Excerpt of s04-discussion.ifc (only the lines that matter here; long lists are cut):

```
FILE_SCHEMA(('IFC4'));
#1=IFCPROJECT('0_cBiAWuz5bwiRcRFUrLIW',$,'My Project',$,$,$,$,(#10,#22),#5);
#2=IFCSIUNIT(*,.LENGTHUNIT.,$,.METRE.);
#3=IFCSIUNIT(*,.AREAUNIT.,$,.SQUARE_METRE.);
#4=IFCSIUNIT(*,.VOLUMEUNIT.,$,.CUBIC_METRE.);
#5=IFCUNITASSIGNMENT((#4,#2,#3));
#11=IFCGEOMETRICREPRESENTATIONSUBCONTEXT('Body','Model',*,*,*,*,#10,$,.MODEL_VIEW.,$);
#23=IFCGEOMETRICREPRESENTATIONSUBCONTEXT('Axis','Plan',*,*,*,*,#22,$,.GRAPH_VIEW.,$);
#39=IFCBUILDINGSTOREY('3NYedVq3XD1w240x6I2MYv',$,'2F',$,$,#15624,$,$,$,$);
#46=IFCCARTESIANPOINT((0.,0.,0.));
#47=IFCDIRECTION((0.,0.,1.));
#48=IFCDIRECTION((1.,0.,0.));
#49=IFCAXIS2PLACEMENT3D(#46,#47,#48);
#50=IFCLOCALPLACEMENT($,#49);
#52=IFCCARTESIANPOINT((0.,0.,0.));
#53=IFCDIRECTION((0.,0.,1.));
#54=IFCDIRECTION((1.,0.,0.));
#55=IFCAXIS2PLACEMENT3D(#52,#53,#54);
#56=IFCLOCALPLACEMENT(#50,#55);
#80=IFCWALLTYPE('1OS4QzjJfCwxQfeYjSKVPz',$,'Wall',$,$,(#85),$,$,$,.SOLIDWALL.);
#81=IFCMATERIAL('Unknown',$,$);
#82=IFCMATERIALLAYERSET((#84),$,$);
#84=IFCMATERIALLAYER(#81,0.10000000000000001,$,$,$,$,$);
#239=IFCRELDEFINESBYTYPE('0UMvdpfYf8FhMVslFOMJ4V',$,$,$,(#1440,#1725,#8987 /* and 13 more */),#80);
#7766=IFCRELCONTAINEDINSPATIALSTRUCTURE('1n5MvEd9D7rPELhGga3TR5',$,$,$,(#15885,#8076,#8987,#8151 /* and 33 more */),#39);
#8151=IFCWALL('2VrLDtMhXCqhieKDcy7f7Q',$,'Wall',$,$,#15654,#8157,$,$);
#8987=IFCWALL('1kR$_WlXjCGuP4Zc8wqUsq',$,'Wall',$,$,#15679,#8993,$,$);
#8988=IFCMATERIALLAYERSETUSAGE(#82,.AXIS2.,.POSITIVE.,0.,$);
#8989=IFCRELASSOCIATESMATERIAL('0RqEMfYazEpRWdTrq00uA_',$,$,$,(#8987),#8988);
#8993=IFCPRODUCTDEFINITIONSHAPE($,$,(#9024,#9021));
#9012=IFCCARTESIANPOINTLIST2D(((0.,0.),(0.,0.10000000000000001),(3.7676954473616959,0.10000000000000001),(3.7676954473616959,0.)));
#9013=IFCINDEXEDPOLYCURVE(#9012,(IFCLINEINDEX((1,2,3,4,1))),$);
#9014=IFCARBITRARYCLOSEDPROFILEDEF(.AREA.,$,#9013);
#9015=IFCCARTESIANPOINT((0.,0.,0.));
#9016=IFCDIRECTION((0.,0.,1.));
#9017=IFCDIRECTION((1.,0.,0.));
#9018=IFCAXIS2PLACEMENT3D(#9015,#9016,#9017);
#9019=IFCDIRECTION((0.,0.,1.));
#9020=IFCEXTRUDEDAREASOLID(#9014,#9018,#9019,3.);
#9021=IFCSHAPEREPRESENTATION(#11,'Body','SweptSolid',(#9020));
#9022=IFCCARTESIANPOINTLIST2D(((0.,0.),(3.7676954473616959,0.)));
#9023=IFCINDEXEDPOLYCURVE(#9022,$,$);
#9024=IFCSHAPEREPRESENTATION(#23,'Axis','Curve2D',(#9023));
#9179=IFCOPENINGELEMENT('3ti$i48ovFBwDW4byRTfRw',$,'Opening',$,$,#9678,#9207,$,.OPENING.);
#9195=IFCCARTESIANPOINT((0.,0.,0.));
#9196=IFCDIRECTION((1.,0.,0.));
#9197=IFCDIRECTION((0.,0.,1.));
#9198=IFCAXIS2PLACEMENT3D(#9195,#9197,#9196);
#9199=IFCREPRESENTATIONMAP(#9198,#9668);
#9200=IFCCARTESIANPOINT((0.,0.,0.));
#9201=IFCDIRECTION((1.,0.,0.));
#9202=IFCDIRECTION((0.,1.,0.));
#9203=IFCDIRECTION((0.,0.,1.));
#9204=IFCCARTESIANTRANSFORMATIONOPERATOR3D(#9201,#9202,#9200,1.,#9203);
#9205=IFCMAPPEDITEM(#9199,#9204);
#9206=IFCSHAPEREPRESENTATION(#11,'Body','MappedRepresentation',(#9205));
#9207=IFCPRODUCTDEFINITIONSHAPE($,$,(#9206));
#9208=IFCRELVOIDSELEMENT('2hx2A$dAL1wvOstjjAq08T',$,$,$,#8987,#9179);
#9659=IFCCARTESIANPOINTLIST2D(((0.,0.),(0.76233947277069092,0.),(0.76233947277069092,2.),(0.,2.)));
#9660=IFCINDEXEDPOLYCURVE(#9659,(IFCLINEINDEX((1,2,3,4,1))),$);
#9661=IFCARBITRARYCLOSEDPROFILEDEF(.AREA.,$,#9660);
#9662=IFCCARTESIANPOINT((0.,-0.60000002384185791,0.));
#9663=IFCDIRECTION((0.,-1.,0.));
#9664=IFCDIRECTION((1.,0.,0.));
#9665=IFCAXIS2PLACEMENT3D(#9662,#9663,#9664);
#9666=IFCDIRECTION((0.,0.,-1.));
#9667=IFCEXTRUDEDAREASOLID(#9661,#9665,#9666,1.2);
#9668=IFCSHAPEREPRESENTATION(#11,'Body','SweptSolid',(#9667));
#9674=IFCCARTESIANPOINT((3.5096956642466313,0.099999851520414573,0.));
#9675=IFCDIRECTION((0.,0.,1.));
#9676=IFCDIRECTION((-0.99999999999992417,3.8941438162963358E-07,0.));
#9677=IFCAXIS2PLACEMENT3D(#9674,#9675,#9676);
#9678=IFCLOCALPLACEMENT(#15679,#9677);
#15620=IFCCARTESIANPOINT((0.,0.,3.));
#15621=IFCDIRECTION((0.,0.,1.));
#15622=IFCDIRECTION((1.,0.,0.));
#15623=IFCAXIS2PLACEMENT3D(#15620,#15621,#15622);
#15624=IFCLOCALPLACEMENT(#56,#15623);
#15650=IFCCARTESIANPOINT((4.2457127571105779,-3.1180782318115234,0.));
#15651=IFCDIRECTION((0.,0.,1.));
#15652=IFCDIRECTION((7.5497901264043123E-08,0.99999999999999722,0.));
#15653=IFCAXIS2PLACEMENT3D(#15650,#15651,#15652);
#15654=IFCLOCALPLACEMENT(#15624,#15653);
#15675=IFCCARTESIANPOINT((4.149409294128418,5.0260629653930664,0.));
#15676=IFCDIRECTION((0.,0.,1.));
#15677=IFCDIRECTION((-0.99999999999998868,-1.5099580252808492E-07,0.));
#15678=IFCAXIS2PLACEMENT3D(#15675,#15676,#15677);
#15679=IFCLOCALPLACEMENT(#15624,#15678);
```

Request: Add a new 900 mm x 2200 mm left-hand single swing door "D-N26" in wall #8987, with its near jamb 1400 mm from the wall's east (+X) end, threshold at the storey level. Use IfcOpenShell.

```python
import numpy as np
import ifcopenshell
import ifcopenshell.api.feature
import ifcopenshell.api.geometry
import ifcopenshell.api.root
import ifcopenshell.api.spatial
import ifcopenshell.geom
import ifcopenshell.util.element
import ifcopenshell.util.placement
import ifcopenshell.util.representation
import ifcopenshell.util.shape
import ifcopenshell.util.unit

model = ifcopenshell.open("s04-discussion.ifc")
unit_scale = ifcopenshell.util.unit.calculate_unit_scale(model)
settings = ifcopenshell.geom.settings()


def volume(element):
    """Net volume in cubic metres, openings subtracted."""
    shape = ifcopenshell.geom.create_shape(settings, element)
    return ifcopenshell.util.shape.get_volume(shape.geometry)


wall = model.by_guid("1kR$_WlXjCGuP4Zc8wqUsq")
storey = ifcopenshell.util.element.get_container(wall, ifc_class="IfcBuildingStorey")
context = ifcopenshell.util.representation.get_context(model, "Model", "Body", "MODEL_VIEW")
before = volume(wall)

width, height, from_end, sill = 0.9, 2.2, 1.4, 0.0  # metres

# The wall runs along its own X axis, and the end named is its -X end.
wall_shape = ifcopenshell.geom.create_shape(settings, wall)
x, y, z = ifcopenshell.util.shape.get_vertices(wall_shape.geometry).T
start = x.min() + from_end
face, thickness = float(y.min()), float(y.max() - y.min())
wall_matrix = ifcopenshell.util.placement.get_local_placement(wall.ObjectPlacement)
level = ifcopenshell.util.placement.get_local_placement(storey.ObjectPlacement)[2, 3]


def in_wall(x, y):
    """Placement at x, y metres in the wall's axes, at sill height."""
    matrix = wall_matrix.copy()
    matrix[:, 3] = wall_matrix @ np.array([x / unit_scale, y / unit_scale, 0.0, 1.0])
    matrix[2, 3] = level + sill / unit_scale
    return matrix


# Opening: a box that overshoots both wall faces by 50 mm.
opening = ifcopenshell.api.root.create_entity(model, ifc_class="IfcOpeningElement", predefined_type="OPENING")
box = ifcopenshell.api.geometry.add_wall_representation(
    model, context=context, length=width, height=height, thickness=thickness + 0.1
)
ifcopenshell.api.geometry.assign_representation(model, product=opening, representation=box)
ifcopenshell.api.geometry.edit_object_placement(model, product=opening, matrix=in_wall(start, face - 0.05), is_si=False)
ifcopenshell.api.feature.add_feature(model, feature=opening, element=wall)

door = ifcopenshell.api.root.create_entity(model, ifc_class="IfcDoor", name="D-N26", predefined_type="DOOR")
door.OverallWidth, door.OverallHeight = width / unit_scale, height / unit_scale
door.OperationType = "SINGLE_SWING_LEFT"
body = ifcopenshell.api.geometry.add_door_representation(
    model,
    context=context,
    overall_width=door.OverallWidth,
    overall_height=door.OverallHeight,
    operation_type="SINGLE_SWING_LEFT",
    lining_properties={"LiningDepth": thickness / unit_scale, "ThresholdDepth": thickness / unit_scale},
)
ifcopenshell.api.geometry.assign_representation(model, product=door, representation=body)
ifcopenshell.api.spatial.assign_container(model, products=[door], relating_structure=storey)
ifcopenshell.api.feature.add_filling(model, opening=opening, element=door)

# The lining spans the wall, so the door starts at the wall face.
ifcopenshell.api.geometry.edit_object_placement(model, product=door, matrix=in_wall(start, face), is_si=False)

after = volume(wall)

print(f"wall volume {before:.3f} -> {after:.3f} m3")

model.write("s04-discussion-out.ifc")
```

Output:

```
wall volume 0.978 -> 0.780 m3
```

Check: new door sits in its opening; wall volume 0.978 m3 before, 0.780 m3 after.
